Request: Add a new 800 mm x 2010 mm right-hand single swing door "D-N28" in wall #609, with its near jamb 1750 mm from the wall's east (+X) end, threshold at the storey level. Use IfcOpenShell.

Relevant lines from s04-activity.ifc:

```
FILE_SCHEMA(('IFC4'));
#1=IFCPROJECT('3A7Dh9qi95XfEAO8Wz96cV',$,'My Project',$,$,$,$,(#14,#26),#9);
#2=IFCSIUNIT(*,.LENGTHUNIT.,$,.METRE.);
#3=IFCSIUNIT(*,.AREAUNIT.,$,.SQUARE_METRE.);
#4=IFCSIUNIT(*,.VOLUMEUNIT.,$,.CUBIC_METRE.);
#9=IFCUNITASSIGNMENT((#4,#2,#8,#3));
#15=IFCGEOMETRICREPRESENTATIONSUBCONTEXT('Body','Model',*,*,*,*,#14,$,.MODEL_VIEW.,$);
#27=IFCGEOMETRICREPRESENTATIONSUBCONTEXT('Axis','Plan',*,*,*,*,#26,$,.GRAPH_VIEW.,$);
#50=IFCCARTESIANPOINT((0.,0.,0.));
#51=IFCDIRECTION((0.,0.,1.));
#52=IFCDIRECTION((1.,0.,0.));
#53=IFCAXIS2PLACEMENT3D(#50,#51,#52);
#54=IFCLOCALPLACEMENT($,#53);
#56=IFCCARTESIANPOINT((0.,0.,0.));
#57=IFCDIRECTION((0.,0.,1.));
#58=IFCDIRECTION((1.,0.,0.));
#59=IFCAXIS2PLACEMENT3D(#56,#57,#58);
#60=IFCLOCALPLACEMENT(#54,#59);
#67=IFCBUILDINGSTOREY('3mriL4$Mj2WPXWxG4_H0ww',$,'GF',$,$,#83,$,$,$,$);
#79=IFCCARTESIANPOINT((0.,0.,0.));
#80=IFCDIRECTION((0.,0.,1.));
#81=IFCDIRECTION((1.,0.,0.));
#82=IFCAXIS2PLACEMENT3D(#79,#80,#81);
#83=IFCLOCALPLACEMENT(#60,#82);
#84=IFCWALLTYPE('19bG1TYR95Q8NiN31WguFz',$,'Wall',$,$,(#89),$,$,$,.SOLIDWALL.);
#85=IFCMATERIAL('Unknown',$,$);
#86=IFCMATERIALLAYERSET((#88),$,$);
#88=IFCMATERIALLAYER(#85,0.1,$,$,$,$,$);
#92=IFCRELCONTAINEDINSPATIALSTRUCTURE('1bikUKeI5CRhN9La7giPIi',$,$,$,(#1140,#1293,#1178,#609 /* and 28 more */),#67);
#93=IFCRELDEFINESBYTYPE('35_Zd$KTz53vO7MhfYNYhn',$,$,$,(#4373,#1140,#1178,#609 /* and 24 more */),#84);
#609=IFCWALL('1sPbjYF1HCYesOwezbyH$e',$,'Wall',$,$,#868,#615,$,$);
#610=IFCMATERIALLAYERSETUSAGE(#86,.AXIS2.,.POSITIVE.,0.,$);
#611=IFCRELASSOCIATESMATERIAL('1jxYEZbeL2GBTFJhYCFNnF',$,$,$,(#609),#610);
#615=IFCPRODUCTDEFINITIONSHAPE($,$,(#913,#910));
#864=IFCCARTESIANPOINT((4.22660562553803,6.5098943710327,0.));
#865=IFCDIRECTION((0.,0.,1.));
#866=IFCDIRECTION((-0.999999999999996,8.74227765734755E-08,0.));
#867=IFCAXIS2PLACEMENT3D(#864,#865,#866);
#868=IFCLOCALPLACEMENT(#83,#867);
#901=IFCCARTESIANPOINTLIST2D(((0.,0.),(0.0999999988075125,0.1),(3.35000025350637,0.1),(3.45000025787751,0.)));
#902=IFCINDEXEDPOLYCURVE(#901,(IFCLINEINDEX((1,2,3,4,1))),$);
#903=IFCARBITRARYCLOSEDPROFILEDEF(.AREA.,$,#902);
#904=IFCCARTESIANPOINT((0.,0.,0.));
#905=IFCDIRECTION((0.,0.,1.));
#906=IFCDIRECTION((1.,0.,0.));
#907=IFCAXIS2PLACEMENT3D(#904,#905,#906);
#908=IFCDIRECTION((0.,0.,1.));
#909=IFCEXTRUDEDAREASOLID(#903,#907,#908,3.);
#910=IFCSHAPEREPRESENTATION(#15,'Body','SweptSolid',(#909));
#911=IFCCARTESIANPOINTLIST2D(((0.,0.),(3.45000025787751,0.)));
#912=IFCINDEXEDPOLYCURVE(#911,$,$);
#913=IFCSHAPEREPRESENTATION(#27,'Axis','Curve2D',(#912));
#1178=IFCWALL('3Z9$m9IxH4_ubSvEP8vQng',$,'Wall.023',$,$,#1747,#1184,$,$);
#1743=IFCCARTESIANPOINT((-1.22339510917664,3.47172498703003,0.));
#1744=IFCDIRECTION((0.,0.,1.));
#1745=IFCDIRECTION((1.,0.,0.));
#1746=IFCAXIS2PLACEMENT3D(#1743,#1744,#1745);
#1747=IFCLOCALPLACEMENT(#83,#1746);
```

```python
import numpy as np
import ifcopenshell
import ifcopenshell.api.feature
import ifcopenshell.api.geometry
import ifcopenshell.api.root
import ifcopenshell.api.spatial
import ifcopenshell.geom
import ifcopenshell.util.element
import ifcopenshell.util.placement
import ifcopenshell.util.representation
import ifcopenshell.util.shape
import ifcopenshell.util.unit

model = ifcopenshell.open("s04-activity.ifc")
unit_scale = ifcopenshell.util.unit.calculate_unit_scale(model)
settings = ifcopenshell.geom.settings()


def volume(element):
    """Net volume in cubic metres, openings subtracted."""
    shape = ifcopenshell.geom.create_shape(settings, element)
    return ifcopenshell.util.shape.get_volume(shape.geometry)


wall = model.by_id(609)
storey = ifcopenshell.util.element.get_container(wall, ifc_class="IfcBuildingStorey")
context = ifcopenshell.util.representation.get_context(model, "Model", "Body", "MODEL_VIEW")
before = volume(wall)

width, height, from_end, sill = 0.8, 2.01, 1.75, 0.0  # metres

# The wall runs along its own X axis, and the end named is its -X end.
wall_shape = ifcopenshell.geom.create_shape(settings, wall)
x, y, z = ifcopenshell.util.shape.get_vertices(wall_shape.geometry).T
start = x.min() + from_end
face, thickness = float(y.min()), float(y.max() - y.min())
wall_matrix = ifcopenshell.util.placement.get_local_placement(wall.ObjectPlacement)
level = ifcopenshell.util.placement.get_local_placement(storey.ObjectPlacement)[2, 3]


def in_wall(x, y):
    """Placement at x, y metres in the wall's axes, at sill height."""
    matrix = wall_matrix.copy()
    matrix[:, 3] = wall_matrix @ np.array([x / unit_scale, y / unit_scale, 0.0, 1.0])
    matrix[2, 3] = level + sill / unit_scale
    return matrix


# Opening: a box that overshoots both wall faces by 50 mm.
opening = ifcopenshell.api.root.create_entity(model, ifc_class="IfcOpeningElement", predefined_type="OPENING")
box = ifcopenshell.api.geometry.add_wall_representation(
    model, context=context, length=width, height=height, thickness=thickness + 0.1
)
ifcopenshell.api.geometry.assign_representation(model, product=opening, representation=box)
ifcopenshell.api.geometry.edit_object_placement(model, product=opening, matrix=in_wall(start, face - 0.05), is_si=False)
ifcopenshell.api.feature.add_feature(model, feature=opening, element=wall)

door = ifcopenshell.api.root.create_entity(model, ifc_class="IfcDoor", name="D-N28", predefined_type="DOOR")
door.OverallWidth, door.OverallHeight = width / unit_scale, height / unit_scale
door.OperationType = "SINGLE_SWING_RIGHT"
body = ifcopenshell.api.geometry.add_door_representation(
    model,
    context=context,
    overall_width=door.OverallWidth,
    overall_height=door.OverallHeight,
    operation_type="SINGLE_SWING_RIGHT",
    lining_properties={"LiningDepth": thickness / unit_scale, "ThresholdDepth": thickness / unit_scale},
)
ifcopenshell.api.geometry.assign_representation(model, product=door, representation=body)
ifcopenshell.api.spatial.assign_container(model, products=[door], relating_structure=storey)
ifcopenshell.api.feature.add_filling(model, opening=opening, element=door)

# The lining spans the wall, so the door starts at the wall face.
ifcopenshell.api.geometry.edit_object_placement(model, product=door, matrix=in_wall(start, face), is_si=False)

after = volume(wall)

print(f"wall volume {before:.3f} -> {after:.3f} m3")

model.write("s04-activity_v2.ifc")
```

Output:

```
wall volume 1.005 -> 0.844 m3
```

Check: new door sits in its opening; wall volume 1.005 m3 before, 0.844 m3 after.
